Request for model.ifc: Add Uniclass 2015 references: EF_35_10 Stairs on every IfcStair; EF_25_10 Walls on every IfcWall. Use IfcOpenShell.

First a look at what the model holds.

```python
import ifcopenshell

model = ifcopenshell.open("model.ifc")
print(model.schema)
print("classifications:", [c.Name for c in model.by_type("IfcClassification")])
for ifc_class in ("IfcDoor", "IfcRoof", "IfcStair", "IfcWall", "IfcWindow"):
    print(ifc_class, len(model.by_type(ifc_class)))
```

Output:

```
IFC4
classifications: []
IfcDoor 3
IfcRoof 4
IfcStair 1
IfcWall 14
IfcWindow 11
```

```python
import ifcopenshell
import ifcopenshell.api.classification

model = ifcopenshell.open("model.ifc")

system = ifcopenshell.api.classification.add_classification(model, classification="Uniclass 2015")

codes = {
    "IfcStair": ("EF_35_10", "Stairs"),
    "IfcWall": ("EF_25_10", "Walls"),
}
for ifc_class, (code, name) in codes.items():
    products = model.by_type(ifc_class)
    ifcopenshell.api.classification.add_reference(
        model, products=products, classification=system, identification=code, name=name
    )
    print(code, len(products))

model.write("model_rev.ifc")
```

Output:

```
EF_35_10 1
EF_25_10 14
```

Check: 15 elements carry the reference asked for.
